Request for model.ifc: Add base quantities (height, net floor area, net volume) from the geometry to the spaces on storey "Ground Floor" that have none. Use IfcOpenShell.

First a look at what the model holds.

```python
import ifcopenshell
import ifcopenshell.util.element
import ifcopenshell.util.unit

model = ifcopenshell.open("model.ifc")
print(model.schema)
for unit_type in ("LENGTHUNIT", "AREAUNIT", "VOLUMEUNIT"):
    print(unit_type, ifcopenshell.util.unit.calculate_unit_scale(model, unit_type))
storey = next(s for s in model.by_type("IfcBuildingStorey") if s.Name == "Ground Floor")
spaces = [e for e in ifcopenshell.util.element.get_decomposition(storey) if e.is_a("IfcSpace")]
for e in sorted(spaces, key=lambda e: e.id()):
    print(e.id(), e.is_a(), e.Name, list(ifcopenshell.util.element.get_psets(e, qtos_only=True)), sep=" | ")
```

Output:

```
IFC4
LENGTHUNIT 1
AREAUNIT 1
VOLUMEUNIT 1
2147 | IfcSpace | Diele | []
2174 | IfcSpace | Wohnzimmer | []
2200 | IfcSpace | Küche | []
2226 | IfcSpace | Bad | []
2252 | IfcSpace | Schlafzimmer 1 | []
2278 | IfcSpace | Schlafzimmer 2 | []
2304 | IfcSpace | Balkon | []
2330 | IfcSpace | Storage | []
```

```python
import ifcopenshell
import ifcopenshell.api.pset
import ifcopenshell.geom
import ifcopenshell.util.element
import ifcopenshell.util.shape
import ifcopenshell.util.unit

model = ifcopenshell.open("model.ifc")
unit_scale = ifcopenshell.util.unit.calculate_unit_scale(model)
area_scale = ifcopenshell.util.unit.calculate_unit_scale(model, "AREAUNIT")
volume_scale = ifcopenshell.util.unit.calculate_unit_scale(model, "VOLUMEUNIT")
settings = ifcopenshell.geom.settings()

storey = next(s for s in model.by_type("IfcBuildingStorey") if s.Name == "Ground Floor")
spaces = [e for e in ifcopenshell.util.element.get_decomposition(storey) if e.is_a("IfcSpace")]

for e in sorted(spaces, key=lambda e: e.id()):
    if ifcopenshell.util.element.get_psets(e, qtos_only=True, should_inherit=False):
        continue
    # Geometry comes back in metres, in the element's own axes.
    shape = ifcopenshell.geom.create_shape(settings, e)
    values = {
        "Height": ifcopenshell.util.shape.get_z(shape.geometry) / unit_scale,
        "NetFloorArea": ifcopenshell.util.shape.get_footprint_area(shape.geometry) / area_scale,
        "NetVolume": ifcopenshell.util.shape.get_volume(shape.geometry) / volume_scale,
    }
    qto = ifcopenshell.api.pset.add_qto(model, product=e, name="Qto_SpaceBaseQuantities")
    ifcopenshell.api.pset.edit_qto(model, qto=qto, properties=values)
    print(e.id(), {k: round(v, 3) for k, v in values.items()})

model.write("model_rev.ifc")
```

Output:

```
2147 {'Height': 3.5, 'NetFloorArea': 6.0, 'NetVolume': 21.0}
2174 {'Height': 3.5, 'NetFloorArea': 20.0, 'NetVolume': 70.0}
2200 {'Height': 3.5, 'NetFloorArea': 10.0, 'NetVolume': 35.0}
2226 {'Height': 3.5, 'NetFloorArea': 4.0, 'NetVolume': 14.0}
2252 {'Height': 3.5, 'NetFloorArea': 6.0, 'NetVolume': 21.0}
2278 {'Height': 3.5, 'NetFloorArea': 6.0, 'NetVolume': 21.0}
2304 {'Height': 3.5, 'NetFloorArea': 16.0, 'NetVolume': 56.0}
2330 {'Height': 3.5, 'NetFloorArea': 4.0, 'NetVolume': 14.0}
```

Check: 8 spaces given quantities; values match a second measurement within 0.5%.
